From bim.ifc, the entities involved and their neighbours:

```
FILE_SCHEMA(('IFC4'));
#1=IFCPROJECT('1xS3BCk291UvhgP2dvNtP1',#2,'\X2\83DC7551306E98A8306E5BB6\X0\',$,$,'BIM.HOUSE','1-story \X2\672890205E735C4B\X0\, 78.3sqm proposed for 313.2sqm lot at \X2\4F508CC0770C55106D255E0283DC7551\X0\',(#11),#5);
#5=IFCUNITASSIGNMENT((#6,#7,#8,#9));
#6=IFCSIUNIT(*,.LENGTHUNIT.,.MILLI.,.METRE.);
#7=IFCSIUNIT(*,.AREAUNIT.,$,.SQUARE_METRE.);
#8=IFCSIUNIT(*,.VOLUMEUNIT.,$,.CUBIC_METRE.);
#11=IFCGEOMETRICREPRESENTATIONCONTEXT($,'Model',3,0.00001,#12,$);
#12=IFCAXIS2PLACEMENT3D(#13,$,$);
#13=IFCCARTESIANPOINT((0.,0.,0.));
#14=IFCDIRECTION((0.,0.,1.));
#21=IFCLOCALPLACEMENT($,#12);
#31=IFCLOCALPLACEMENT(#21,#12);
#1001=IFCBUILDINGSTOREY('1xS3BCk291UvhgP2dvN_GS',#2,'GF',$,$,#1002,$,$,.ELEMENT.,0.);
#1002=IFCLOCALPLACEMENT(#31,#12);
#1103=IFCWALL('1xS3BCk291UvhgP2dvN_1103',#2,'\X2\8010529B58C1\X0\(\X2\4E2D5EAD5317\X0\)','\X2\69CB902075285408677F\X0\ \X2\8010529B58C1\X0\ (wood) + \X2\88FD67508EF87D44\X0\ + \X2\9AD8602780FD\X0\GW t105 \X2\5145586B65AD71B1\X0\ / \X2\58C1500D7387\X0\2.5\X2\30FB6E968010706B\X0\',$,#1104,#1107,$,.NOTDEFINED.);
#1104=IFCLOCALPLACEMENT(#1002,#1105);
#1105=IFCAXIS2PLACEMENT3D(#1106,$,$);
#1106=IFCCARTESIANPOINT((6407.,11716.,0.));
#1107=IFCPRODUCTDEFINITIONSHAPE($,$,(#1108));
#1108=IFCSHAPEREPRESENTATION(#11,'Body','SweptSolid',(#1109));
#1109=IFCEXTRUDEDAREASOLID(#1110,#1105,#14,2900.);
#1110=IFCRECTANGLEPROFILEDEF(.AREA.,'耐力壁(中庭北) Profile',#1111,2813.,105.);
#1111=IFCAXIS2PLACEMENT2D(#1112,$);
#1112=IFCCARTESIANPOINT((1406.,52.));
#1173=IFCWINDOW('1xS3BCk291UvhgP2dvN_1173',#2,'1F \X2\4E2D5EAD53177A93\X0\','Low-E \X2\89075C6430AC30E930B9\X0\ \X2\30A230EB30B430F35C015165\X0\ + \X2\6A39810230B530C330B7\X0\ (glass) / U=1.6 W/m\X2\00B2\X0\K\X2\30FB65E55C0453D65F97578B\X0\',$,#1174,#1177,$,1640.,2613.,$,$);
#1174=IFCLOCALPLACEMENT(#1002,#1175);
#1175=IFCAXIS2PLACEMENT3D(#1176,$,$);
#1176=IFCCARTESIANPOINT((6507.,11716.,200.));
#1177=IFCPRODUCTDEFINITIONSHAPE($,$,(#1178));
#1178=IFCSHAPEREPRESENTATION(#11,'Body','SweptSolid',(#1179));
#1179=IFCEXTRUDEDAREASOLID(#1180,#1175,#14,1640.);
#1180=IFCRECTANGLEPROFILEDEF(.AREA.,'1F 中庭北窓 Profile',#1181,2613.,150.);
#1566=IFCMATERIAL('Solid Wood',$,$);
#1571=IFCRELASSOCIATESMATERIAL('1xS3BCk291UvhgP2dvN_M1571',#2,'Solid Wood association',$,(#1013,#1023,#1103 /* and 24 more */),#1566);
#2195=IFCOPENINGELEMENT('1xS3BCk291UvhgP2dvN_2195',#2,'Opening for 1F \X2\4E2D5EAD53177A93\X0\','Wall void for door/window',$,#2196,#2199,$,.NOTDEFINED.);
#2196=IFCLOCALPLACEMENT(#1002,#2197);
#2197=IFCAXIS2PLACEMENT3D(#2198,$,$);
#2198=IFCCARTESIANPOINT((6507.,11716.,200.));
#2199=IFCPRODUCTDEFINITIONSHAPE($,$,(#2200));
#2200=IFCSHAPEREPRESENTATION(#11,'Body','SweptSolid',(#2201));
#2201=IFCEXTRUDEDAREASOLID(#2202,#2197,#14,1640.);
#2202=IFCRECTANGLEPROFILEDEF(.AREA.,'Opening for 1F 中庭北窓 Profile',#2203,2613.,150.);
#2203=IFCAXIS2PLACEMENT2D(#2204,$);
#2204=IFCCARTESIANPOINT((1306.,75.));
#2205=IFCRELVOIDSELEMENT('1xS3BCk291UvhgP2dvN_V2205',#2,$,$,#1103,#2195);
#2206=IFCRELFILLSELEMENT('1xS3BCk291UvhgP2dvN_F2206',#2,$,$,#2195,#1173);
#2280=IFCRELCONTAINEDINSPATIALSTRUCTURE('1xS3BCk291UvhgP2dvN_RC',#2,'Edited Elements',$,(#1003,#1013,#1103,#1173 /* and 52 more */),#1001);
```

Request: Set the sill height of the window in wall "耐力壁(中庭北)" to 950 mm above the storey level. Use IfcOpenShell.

```python
import numpy as np
import ifcopenshell
import ifcopenshell.api.geometry
import ifcopenshell.geom
import ifcopenshell.util.element
import ifcopenshell.util.placement
import ifcopenshell.util.shape
import ifcopenshell.util.unit

model = ifcopenshell.open("bim.ifc")
unit_scale = ifcopenshell.util.unit.calculate_unit_scale(model)

window = model.by_guid("1xS3BCk291UvhgP2dvN_1173")
opening = window.FillsVoids[0].RelatingOpeningElement
storey = ifcopenshell.util.element.get_container(window, ifc_class="IfcBuildingStorey")
level = ifcopenshell.util.placement.get_local_placement(storey.ObjectPlacement)[2, 3]

# The opening's origin need not be at the sill, so measure its lowest point.
shape = ifcopenshell.geom.create_shape(ifcopenshell.geom.settings(), opening)
bottom = ifcopenshell.util.shape.get_shape_bottom_elevation(shape, shape.geometry) / unit_scale
dz = level + 0.95 / unit_scale - bottom

shift = np.array([0.0, 0.0, dz])
# The window is not placed relative to its opening, so move both.
for product in (opening, window):
    matrix = ifcopenshell.util.placement.get_local_placement(product.ObjectPlacement)
    matrix[:3, 3] += shift
    ifcopenshell.api.geometry.edit_object_placement(model, product=product, matrix=matrix, is_si=False)

print(f"moved by {dz * unit_scale:+.3f} m")

model.write("bim_edited.ifc")
```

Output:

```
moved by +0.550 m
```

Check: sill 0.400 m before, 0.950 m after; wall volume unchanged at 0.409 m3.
